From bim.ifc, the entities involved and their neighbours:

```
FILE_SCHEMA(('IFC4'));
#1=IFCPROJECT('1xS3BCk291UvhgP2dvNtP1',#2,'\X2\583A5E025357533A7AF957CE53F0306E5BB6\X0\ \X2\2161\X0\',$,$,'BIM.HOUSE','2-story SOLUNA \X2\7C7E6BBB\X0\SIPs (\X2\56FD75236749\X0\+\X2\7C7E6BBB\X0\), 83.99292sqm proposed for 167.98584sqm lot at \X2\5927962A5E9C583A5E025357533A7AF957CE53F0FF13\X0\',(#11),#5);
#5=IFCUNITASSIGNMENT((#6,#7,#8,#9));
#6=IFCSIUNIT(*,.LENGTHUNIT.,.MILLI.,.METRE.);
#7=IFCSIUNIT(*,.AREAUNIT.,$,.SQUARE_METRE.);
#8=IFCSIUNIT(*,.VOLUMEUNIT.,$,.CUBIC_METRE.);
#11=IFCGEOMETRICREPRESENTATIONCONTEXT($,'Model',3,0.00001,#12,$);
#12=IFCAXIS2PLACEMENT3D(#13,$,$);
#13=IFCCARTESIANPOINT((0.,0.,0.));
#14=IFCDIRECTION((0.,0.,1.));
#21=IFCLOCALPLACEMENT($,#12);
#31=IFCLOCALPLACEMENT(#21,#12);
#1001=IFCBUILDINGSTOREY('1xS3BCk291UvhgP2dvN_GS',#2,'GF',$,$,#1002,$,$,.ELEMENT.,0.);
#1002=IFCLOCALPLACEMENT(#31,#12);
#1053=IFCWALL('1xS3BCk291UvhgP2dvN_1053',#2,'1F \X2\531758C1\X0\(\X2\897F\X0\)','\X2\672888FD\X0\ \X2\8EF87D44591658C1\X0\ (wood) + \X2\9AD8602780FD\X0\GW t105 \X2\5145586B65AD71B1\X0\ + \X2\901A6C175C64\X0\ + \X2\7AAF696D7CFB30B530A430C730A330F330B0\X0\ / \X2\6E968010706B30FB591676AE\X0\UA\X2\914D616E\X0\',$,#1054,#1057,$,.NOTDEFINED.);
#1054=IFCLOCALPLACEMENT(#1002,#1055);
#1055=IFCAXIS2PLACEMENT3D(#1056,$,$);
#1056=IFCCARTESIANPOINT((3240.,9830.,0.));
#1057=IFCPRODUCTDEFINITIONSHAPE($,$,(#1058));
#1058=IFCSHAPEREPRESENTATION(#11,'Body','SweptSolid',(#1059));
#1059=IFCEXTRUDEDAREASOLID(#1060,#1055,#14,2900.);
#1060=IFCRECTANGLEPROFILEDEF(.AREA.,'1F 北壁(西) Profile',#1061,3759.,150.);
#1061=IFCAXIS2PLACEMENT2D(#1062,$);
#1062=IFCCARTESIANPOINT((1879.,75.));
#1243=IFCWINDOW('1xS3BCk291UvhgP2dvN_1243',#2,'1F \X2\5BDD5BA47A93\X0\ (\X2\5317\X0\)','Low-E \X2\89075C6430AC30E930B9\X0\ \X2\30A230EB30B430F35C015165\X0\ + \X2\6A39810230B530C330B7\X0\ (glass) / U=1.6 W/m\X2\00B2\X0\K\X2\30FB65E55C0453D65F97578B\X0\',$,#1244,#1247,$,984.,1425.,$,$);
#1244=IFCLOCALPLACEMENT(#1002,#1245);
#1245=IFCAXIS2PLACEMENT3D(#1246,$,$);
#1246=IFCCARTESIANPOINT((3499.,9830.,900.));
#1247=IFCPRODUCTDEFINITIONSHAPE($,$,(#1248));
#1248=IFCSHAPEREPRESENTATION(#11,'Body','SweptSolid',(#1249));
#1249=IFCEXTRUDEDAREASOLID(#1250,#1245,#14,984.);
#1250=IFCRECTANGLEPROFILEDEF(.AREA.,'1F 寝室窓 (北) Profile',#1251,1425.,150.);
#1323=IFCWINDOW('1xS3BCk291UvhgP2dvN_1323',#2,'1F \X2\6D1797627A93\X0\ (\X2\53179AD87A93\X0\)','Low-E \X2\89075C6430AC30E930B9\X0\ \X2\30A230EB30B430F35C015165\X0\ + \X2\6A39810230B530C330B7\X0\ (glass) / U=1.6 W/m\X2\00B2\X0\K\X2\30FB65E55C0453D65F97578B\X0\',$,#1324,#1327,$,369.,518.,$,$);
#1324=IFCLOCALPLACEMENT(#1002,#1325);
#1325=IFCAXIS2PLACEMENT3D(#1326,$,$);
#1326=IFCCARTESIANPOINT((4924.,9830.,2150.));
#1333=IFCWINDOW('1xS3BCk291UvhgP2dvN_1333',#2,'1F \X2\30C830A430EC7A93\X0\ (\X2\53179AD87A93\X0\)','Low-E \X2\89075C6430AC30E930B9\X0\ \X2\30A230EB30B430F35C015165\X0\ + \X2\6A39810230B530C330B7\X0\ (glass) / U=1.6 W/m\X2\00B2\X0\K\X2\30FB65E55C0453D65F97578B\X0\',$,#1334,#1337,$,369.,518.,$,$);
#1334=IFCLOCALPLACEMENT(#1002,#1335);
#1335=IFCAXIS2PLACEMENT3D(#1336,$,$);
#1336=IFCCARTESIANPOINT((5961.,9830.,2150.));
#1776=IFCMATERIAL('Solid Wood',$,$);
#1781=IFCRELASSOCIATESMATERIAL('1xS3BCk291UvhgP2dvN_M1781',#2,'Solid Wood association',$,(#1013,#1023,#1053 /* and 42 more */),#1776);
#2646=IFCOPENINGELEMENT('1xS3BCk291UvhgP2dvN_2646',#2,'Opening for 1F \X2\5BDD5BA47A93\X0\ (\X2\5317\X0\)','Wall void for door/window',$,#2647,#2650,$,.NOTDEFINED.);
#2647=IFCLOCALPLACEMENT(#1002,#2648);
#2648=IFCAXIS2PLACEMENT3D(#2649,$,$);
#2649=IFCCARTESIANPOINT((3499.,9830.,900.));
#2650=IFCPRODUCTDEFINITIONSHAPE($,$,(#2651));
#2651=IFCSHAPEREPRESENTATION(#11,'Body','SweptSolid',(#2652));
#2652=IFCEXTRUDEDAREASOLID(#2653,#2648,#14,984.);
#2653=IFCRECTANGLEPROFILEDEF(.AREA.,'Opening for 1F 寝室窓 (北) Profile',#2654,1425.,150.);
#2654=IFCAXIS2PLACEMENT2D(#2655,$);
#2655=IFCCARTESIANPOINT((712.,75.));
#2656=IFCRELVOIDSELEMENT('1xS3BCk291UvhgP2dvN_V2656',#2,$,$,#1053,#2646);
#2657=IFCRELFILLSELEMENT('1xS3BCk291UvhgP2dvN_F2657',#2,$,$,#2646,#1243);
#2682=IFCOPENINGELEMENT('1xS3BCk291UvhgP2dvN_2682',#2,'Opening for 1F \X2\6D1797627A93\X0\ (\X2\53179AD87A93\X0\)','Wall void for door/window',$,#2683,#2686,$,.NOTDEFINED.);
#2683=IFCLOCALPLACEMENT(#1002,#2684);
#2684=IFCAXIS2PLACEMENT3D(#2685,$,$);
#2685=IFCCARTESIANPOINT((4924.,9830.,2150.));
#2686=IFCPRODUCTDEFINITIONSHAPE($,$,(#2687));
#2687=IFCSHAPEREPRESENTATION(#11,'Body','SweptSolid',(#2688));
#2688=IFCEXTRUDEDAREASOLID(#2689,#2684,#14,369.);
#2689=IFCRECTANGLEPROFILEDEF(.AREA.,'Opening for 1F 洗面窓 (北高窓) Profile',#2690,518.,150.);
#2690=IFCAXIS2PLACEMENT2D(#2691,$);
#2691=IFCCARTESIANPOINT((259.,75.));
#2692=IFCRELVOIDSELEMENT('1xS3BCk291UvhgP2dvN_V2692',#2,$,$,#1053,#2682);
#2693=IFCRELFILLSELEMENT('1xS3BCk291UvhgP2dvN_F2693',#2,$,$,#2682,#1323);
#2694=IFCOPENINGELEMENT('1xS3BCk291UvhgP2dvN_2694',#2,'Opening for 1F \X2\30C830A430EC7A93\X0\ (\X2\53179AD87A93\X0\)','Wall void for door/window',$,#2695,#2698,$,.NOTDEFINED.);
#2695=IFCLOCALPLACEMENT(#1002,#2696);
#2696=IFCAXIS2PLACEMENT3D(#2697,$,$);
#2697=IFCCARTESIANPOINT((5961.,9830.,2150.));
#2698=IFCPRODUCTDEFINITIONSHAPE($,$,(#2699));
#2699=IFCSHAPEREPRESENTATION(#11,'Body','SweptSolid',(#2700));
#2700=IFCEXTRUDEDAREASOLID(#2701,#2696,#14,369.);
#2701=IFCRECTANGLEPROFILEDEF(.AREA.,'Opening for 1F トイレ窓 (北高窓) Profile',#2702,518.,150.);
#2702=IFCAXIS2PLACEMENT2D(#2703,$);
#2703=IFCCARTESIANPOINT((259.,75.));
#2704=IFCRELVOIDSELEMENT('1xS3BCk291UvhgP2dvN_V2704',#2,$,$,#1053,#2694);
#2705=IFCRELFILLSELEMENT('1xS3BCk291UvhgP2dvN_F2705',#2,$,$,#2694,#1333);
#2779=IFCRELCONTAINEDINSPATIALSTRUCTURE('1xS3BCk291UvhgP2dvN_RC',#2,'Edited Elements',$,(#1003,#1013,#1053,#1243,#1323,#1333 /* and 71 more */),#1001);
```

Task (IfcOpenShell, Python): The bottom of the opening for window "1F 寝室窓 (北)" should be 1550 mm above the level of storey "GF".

```python
import numpy as np
import ifcopenshell
import ifcopenshell.api.geometry
import ifcopenshell.geom
import ifcopenshell.util.element
import ifcopenshell.util.placement
import ifcopenshell.util.shape
import ifcopenshell.util.unit

model = ifcopenshell.open("bim.ifc")
unit_scale = ifcopenshell.util.unit.calculate_unit_scale(model)

window = model.by_guid("1xS3BCk291UvhgP2dvN_1243")
opening = window.FillsVoids[0].RelatingOpeningElement
storey = ifcopenshell.util.element.get_container(window, ifc_class="IfcBuildingStorey")
level = ifcopenshell.util.placement.get_local_placement(storey.ObjectPlacement)[2, 3]

# The opening's origin need not be at the sill, so measure its lowest point.
shape = ifcopenshell.geom.create_shape(ifcopenshell.geom.settings(), opening)
bottom = ifcopenshell.util.shape.get_shape_bottom_elevation(shape, shape.geometry) / unit_scale
dz = level + 1.55 / unit_scale - bottom

shift = np.array([0.0, 0.0, dz])
# The window is not placed relative to its opening, so move both.
for product in (opening, window):
    matrix = ifcopenshell.util.placement.get_local_placement(product.ObjectPlacement)
    matrix[:3, 3] += shift
    ifcopenshell.api.geometry.edit_object_placement(model, product=product, matrix=matrix, is_si=False)

print(f"moved by {dz * unit_scale:+.3f} m")

model.write("bim_v2.ifc")
```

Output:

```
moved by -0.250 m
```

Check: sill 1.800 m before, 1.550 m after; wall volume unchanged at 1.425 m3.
